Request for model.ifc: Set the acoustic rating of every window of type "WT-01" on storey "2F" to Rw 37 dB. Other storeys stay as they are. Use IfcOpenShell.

First a look at what the model holds.

```python
import ifcopenshell
import ifcopenshell.util.element

model = ifcopenshell.open("model.ifc")
print(model.schema)
storey = next(s for s in model.by_type("IfcBuildingStorey") if s.Name == "2F")
windows = [e for e in ifcopenshell.util.element.get_decomposition(storey) if e.is_a("IfcWindow")]
seen = {}
for e in windows:
    element_type = ifcopenshell.util.element.get_type(e)
    key = (element_type.Name if element_type != e and element_type else None, ifcopenshell.util.element.get_pset(e, "Pset_WindowCommon", "AcousticRating"))
    seen[key] = seen.get(key, 0) + 1
for (name, value), count in sorted(seen.items(), key=str):
    print(count, "x", name, "|", value)
```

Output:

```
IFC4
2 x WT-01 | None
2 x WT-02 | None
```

```python
import ifcopenshell
import ifcopenshell.api.pset
import ifcopenshell.util.element

model = ifcopenshell.open("model.ifc")

storey = next(s for s in model.by_type("IfcBuildingStorey") if s.Name == "2F")
windows = [e for e in ifcopenshell.util.element.get_decomposition(storey) if e.is_a("IfcWindow")]

count = 0
for e in windows:
    element_type = ifcopenshell.util.element.get_type(e)
    if element_type in (None, e) or element_type.Name != "WT-01":
        continue
    # add_pset returns the element's existing set when there is one.
    pset = ifcopenshell.api.pset.add_pset(model, product=e, name="Pset_WindowCommon")
    ifcopenshell.api.pset.edit_pset(model, pset=pset, properties={"AcousticRating": "Rw 37 dB"})
    count += 1

print(count, "windows updated")

model.write("model_edited.ifc")
```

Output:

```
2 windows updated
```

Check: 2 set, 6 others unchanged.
